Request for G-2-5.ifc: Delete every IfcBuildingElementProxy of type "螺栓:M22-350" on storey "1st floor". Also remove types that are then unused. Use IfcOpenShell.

First a look at what the model holds.

```python
import ifcopenshell
import ifcopenshell.util.element

model = ifcopenshell.open("G-2-5.ifc")
print(model.schema)
storey = next(s for s in model.by_type("IfcBuildingStorey") if s.Name == "1st floor")
proxies = [e for e in ifcopenshell.util.element.get_decomposition(storey) if e.is_a("IfcBuildingElementProxy")]
seen = {}
for e in proxies:
    element_type = ifcopenshell.util.element.get_type(e)
    name = element_type.Name if element_type not in (None, e) else None
    seen[name] = seen.get(name, 0) + 1
for name, count in sorted(seen.items(), key=str):
    print(count, "x", name)
```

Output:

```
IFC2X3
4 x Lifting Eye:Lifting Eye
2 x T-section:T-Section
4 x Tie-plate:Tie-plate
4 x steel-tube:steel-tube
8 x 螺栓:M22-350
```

```python
import ifcopenshell
import ifcopenshell.api.root
import ifcopenshell.util.element

model = ifcopenshell.open("G-2-5.ifc")

storey = next(s for s in model.by_type("IfcBuildingStorey") if s.Name == "1st floor")
proxies = [e for e in ifcopenshell.util.element.get_decomposition(storey) if e.is_a("IfcBuildingElementProxy")]
targets = [e for e in proxies if (t := ifcopenshell.util.element.get_type(e)) not in (None, e) and t.Name == "螺栓:M22-350"]
types = {ifcopenshell.util.element.get_type(e) for e in targets} - {None, *targets}

for e in targets:
    ifcopenshell.api.root.remove_product(model, product=e)
print(len(targets), "removed")

unused = [t for t in types if not ifcopenshell.util.element.get_types(t)]
for t in unused:
    ifcopenshell.api.root.remove_product(model, product=t)
print(len(unused), "unused types removed")

model.write("G-2-5_updated.ifc")
```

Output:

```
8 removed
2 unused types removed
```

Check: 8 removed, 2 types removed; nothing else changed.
